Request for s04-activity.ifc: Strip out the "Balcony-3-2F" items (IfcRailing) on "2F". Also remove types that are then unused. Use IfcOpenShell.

First a look at what the model holds.

```python
import ifcopenshell
import ifcopenshell.util.element

model = ifcopenshell.open("s04-activity.ifc")
print(model.schema)
storey = next(s for s in model.by_type("IfcBuildingStorey") if s.Name == "2F")
railings = [e for e in ifcopenshell.util.element.get_decomposition(storey) if e.is_a("IfcRailing")]
seen = {}
for e in railings:
    element_type = ifcopenshell.util.element.get_type(e)
    name = element_type.Name if element_type not in (None, e) else None
    seen[name] = seen.get(name, 0) + 1
for name, count in sorted(seen.items(), key=str):
    print(count, "x", name)
```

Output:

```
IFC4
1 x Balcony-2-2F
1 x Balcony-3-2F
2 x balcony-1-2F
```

```python
import ifcopenshell
import ifcopenshell.api.root
import ifcopenshell.util.element

model = ifcopenshell.open("s04-activity.ifc")

storey = next(s for s in model.by_type("IfcBuildingStorey") if s.Name == "2F")
railings = [e for e in ifcopenshell.util.element.get_decomposition(storey) if e.is_a("IfcRailing")]
targets = [e for e in railings if (t := ifcopenshell.util.element.get_type(e)) not in (None, e) and t.Name == "Balcony-3-2F"]
types = {ifcopenshell.util.element.get_type(e) for e in targets} - {None, *targets}

for e in targets:
    ifcopenshell.api.root.remove_product(model, product=e)
print(len(targets), "removed")

unused = [t for t in types if not ifcopenshell.util.element.get_types(t)]
for t in unused:
    ifcopenshell.api.root.remove_product(model, product=t)
print(len(unused), "unused types removed")

model.write("s04-activity-out.ifc")
```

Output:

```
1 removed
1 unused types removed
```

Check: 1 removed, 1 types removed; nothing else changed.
